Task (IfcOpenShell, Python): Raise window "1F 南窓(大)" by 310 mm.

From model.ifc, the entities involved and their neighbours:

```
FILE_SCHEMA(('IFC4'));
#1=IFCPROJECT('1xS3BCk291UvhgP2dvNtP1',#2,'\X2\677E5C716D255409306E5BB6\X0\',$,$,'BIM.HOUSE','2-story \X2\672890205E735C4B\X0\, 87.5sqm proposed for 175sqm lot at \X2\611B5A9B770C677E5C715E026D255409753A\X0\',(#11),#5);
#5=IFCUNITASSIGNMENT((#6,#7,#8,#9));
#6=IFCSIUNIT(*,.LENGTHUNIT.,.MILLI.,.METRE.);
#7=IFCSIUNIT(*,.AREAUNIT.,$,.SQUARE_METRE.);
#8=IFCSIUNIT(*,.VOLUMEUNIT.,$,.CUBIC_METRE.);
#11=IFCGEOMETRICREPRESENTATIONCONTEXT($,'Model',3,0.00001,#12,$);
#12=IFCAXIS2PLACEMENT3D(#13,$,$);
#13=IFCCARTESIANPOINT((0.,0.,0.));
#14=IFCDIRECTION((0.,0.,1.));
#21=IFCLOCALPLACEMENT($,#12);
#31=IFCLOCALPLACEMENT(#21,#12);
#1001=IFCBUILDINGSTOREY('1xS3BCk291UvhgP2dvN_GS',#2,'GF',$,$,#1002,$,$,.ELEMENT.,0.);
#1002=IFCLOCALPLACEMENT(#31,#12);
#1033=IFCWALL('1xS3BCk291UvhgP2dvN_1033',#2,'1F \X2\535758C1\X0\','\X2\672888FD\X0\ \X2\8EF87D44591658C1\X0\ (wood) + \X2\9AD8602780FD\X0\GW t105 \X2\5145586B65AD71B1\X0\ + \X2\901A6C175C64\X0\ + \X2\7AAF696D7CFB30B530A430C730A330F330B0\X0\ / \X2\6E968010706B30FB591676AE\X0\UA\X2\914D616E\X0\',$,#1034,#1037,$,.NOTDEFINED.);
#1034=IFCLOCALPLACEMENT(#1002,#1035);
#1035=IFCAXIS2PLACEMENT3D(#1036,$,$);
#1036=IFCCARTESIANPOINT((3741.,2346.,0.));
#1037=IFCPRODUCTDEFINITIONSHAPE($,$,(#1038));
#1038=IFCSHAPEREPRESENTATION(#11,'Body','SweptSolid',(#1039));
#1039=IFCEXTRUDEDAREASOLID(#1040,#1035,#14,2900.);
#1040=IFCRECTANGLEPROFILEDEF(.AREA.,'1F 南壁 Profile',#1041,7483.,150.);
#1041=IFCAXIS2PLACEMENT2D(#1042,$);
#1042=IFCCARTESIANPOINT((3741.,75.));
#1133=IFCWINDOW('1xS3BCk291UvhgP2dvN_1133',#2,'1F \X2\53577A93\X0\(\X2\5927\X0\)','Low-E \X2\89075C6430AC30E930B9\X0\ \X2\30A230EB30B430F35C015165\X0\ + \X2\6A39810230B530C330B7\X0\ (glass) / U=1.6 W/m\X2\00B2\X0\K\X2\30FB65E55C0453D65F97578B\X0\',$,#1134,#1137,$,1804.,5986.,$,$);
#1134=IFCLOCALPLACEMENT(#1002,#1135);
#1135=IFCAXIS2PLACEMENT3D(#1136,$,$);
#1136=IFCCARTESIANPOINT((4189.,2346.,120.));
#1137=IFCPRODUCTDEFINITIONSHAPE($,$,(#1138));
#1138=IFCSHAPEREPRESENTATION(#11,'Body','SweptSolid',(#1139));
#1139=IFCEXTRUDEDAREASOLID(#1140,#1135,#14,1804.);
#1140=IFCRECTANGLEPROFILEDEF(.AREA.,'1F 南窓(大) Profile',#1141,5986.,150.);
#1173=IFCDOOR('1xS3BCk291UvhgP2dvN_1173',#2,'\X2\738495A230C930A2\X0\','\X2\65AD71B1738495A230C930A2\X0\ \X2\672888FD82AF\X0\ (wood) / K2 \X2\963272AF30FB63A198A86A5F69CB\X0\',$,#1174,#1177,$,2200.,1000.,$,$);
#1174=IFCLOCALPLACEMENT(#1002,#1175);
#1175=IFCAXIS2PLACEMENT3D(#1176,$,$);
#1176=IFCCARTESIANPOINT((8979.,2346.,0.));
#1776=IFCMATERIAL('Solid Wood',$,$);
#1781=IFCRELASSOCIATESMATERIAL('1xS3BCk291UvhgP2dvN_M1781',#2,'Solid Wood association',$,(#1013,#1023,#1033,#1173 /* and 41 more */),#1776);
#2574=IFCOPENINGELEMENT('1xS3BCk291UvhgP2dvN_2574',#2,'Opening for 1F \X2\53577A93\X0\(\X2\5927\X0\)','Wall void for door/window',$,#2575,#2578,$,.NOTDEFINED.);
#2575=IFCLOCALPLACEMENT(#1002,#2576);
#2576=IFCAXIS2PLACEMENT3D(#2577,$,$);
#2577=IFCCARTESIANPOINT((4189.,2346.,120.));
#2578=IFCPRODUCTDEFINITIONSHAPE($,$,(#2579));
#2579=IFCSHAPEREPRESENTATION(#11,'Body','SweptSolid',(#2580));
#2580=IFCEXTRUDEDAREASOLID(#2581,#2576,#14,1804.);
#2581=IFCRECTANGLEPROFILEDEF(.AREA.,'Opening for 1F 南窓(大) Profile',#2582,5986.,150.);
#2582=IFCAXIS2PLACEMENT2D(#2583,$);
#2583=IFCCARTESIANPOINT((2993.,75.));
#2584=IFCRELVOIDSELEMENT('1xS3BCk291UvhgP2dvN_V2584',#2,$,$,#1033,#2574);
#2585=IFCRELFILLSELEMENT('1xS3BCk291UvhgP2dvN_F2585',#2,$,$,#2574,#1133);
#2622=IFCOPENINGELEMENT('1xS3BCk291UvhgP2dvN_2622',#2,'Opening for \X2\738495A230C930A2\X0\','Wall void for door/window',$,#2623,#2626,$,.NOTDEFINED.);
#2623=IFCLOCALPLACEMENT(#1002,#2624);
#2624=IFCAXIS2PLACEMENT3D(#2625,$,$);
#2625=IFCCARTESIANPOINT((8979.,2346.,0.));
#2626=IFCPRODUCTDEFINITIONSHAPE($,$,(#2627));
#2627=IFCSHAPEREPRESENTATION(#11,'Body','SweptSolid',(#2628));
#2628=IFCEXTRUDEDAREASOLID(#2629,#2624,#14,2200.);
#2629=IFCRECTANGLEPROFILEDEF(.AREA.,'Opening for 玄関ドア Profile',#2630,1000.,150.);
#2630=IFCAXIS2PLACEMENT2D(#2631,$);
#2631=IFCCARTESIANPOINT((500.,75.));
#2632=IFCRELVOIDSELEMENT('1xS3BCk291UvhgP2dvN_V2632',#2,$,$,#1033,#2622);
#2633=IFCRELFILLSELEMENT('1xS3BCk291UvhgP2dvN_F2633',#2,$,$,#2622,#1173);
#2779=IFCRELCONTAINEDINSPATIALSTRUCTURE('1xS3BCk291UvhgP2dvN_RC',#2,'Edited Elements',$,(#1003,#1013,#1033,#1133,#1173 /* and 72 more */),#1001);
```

```python
import numpy as np
import ifcopenshell
import ifcopenshell.api.geometry
import ifcopenshell.util.placement
import ifcopenshell.util.unit

model = ifcopenshell.open("model.ifc")
unit_scale = ifcopenshell.util.unit.calculate_unit_scale(model)

window = model.by_guid("1xS3BCk291UvhgP2dvN_1133")
opening = window.FillsVoids[0].RelatingOpeningElement
dz = 310.0

shift = np.array([0.0, 0.0, dz])
# The window is not placed relative to its opening, so move both.
for product in (opening, window):
    matrix = ifcopenshell.util.placement.get_local_placement(product.ObjectPlacement)
    matrix[:3, 3] += shift
    ifcopenshell.api.geometry.edit_object_placement(model, product=product, matrix=matrix, is_si=False)

print(f"moved by {dz * unit_scale:+.3f} m")

model.write("model_rev.ifc")
```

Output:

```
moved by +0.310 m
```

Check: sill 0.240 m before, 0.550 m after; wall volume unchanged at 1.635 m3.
